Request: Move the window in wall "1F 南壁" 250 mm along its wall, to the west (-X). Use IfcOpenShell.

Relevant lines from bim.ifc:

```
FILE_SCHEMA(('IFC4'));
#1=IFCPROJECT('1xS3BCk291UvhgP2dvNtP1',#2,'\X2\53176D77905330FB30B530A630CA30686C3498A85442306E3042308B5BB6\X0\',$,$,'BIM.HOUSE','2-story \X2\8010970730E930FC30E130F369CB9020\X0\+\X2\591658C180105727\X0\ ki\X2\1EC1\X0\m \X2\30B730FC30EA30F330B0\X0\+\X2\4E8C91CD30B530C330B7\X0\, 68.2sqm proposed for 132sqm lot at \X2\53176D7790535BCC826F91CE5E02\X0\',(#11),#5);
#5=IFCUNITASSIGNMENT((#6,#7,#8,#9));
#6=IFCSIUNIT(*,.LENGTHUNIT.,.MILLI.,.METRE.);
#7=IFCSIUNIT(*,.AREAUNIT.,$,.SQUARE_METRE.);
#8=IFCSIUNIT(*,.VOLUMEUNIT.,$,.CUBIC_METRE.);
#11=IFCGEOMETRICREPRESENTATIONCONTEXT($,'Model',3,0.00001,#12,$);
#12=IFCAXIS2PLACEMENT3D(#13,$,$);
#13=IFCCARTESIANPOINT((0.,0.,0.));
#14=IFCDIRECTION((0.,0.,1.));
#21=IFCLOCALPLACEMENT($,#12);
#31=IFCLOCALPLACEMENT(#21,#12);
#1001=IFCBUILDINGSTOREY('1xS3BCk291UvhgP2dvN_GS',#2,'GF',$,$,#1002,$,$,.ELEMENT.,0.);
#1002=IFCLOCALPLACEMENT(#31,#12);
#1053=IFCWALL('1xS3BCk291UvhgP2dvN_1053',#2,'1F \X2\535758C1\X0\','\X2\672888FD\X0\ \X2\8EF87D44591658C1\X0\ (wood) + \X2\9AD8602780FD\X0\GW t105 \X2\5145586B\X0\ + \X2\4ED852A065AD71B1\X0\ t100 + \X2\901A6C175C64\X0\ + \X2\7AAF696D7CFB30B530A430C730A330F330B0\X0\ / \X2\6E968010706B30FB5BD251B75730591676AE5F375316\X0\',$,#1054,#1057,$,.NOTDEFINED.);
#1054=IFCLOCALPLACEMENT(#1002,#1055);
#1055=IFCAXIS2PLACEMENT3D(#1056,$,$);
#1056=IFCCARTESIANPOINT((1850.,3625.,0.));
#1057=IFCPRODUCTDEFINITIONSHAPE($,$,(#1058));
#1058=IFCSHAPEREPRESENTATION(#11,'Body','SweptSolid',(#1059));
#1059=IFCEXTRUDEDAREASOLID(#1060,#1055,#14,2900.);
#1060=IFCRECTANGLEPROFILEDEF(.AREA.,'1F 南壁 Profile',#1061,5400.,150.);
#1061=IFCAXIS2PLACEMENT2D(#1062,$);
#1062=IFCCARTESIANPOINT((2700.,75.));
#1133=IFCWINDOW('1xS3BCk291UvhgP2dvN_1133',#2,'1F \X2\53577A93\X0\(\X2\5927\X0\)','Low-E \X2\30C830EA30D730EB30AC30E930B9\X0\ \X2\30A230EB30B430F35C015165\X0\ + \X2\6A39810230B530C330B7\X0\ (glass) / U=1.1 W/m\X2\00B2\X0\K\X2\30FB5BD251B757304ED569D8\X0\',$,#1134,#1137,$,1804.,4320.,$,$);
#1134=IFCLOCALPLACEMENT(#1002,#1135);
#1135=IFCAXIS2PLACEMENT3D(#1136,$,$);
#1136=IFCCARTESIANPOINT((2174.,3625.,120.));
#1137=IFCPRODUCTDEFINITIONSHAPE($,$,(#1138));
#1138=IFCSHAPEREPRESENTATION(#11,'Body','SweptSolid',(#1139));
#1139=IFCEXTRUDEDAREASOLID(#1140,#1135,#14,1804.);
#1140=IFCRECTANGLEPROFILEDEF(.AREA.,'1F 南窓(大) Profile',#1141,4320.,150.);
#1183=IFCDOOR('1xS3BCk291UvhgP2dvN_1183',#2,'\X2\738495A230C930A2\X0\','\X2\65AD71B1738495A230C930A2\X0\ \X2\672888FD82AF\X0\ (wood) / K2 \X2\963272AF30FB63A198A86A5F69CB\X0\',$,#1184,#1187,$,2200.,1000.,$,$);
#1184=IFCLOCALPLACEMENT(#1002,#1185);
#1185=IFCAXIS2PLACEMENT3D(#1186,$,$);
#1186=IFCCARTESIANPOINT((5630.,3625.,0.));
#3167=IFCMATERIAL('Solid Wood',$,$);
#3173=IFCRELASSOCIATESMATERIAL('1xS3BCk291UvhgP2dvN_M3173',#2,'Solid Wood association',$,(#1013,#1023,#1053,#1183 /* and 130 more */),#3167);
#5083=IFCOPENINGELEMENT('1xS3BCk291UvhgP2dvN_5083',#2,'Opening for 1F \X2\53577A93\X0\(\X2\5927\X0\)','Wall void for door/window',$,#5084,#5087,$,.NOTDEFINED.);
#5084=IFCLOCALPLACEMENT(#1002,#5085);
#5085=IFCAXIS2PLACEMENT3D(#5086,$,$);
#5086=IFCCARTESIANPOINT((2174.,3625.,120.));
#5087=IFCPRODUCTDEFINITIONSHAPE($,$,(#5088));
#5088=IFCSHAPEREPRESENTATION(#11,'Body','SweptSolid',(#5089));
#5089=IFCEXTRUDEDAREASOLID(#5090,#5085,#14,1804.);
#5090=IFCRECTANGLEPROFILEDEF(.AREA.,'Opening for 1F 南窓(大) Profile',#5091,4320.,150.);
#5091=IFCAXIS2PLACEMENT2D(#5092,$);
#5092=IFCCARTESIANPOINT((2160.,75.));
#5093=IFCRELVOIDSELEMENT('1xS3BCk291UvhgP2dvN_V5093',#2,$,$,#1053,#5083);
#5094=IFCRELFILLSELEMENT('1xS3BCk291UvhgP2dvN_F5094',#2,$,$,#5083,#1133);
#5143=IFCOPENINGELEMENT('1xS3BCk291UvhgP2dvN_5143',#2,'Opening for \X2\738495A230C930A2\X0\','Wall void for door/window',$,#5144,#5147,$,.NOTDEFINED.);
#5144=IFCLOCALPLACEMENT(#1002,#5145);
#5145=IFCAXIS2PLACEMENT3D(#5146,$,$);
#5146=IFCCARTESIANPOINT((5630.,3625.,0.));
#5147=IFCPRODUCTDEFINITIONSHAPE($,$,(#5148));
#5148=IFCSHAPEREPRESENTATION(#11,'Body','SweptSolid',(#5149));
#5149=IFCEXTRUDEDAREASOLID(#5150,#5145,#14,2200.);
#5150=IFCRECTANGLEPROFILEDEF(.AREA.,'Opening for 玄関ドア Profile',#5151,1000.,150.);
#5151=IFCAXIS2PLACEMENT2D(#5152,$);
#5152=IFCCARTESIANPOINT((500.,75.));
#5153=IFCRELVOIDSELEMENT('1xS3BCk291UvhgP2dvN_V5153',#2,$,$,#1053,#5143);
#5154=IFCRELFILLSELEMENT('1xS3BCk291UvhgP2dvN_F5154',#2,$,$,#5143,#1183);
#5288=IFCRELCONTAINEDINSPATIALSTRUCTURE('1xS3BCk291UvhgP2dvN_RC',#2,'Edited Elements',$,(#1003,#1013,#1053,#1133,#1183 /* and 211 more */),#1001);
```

```python
import ifcopenshell
import ifcopenshell.api.geometry
import ifcopenshell.util.placement
import ifcopenshell.util.unit

model = ifcopenshell.open("bim.ifc")
unit_scale = ifcopenshell.util.unit.calculate_unit_scale(model)

window = model.by_id(1133)
opening = window.FillsVoids[0].RelatingOpeningElement
wall = opening.VoidsElements[0].RelatingBuildingElement

wall_matrix = ifcopenshell.util.placement.get_local_placement(wall.ObjectPlacement)
shift = wall_matrix[:3, 0] * -0.25 / unit_scale
before = ifcopenshell.util.placement.get_local_placement(window.ObjectPlacement)[:3, 3].copy()

# The window is not placed relative to its opening, so move both.
for product in (opening, window):
    matrix = ifcopenshell.util.placement.get_local_placement(product.ObjectPlacement)
    matrix[:3, 3] += shift
    ifcopenshell.api.geometry.edit_object_placement(model, product=product, matrix=matrix, is_si=False)

after = ifcopenshell.util.placement.get_local_placement(window.ObjectPlacement)[:3, 3]
print("window moved by", (after - before).round(3) + 0.0)

model.write("bim_edited.ifc")
```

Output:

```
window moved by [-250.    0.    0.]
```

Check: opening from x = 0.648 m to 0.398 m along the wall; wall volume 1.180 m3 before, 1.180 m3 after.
